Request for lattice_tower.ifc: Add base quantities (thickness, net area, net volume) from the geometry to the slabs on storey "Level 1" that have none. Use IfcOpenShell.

First a look at what the model holds.

```python
import ifcopenshell
import ifcopenshell.util.element
import ifcopenshell.util.unit

model = ifcopenshell.open("lattice_tower.ifc")
print(model.schema)
for unit_type in ("LENGTHUNIT", "AREAUNIT", "VOLUMEUNIT"):
    print(unit_type, ifcopenshell.util.unit.calculate_unit_scale(model, unit_type))
storey = next(s for s in model.by_type("IfcBuildingStorey") if s.Name == "Level 1")
slabs = [e for e in ifcopenshell.util.element.get_decomposition(storey) if e.is_a("IfcSlab")]
for e in sorted(slabs, key=lambda e: e.id()):
    print(e.id(), e.is_a(), e.Name, list(ifcopenshell.util.element.get_psets(e, qtos_only=True)), sep=" | ")
```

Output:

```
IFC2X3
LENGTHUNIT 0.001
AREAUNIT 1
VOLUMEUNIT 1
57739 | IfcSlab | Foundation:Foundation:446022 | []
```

```python
import ifcopenshell
import ifcopenshell.api.pset
import ifcopenshell.geom
import ifcopenshell.util.element
import ifcopenshell.util.shape
import ifcopenshell.util.unit

model = ifcopenshell.open("lattice_tower.ifc")
unit_scale = ifcopenshell.util.unit.calculate_unit_scale(model)
area_scale = ifcopenshell.util.unit.calculate_unit_scale(model, "AREAUNIT")
volume_scale = ifcopenshell.util.unit.calculate_unit_scale(model, "VOLUMEUNIT")
settings = ifcopenshell.geom.settings()

storey = next(s for s in model.by_type("IfcBuildingStorey") if s.Name == "Level 1")
slabs = [e for e in ifcopenshell.util.element.get_decomposition(storey) if e.is_a("IfcSlab")]

for e in sorted(slabs, key=lambda e: e.id()):
    if ifcopenshell.util.element.get_psets(e, qtos_only=True, should_inherit=False):
        continue
    # Geometry comes back in metres, in the element's own axes.
    shape = ifcopenshell.geom.create_shape(settings, e)
    values = {
        "Width": ifcopenshell.util.shape.get_z(shape.geometry) / unit_scale,
        "NetArea": ifcopenshell.util.shape.get_footprint_area(shape.geometry) / area_scale,
        "NetVolume": ifcopenshell.util.shape.get_volume(shape.geometry) / volume_scale,
    }
    qto = ifcopenshell.api.pset.add_qto(model, product=e, name="BaseQuantities")
    ifcopenshell.api.pset.edit_qto(model, qto=qto, properties=values)
    print(e.id(), {k: round(v, 3) for k, v in values.items()})

model.write("lattice_tower_updated.ifc")
```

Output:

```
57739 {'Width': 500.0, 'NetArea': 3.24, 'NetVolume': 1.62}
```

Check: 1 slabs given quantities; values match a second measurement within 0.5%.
